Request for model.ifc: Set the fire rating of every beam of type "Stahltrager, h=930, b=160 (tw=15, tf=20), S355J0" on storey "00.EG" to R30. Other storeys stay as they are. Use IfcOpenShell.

First a look at what the model holds.

```python
import ifcopenshell
import ifcopenshell.util.element

model = ifcopenshell.open("model.ifc")
print(model.schema)
storey = next(s for s in model.by_type("IfcBuildingStorey") if s.Name == "00.EG")
beams = [e for e in ifcopenshell.util.element.get_decomposition(storey) if e.is_a("IfcBeam")]
seen = {}
for e in beams:
    element_type = ifcopenshell.util.element.get_type(e)
    key = (element_type.Name if element_type != e and element_type else None, ifcopenshell.util.element.get_pset(e, "Pset_BeamCommon", "FireRating"))
    seen[key] = seen.get(key, 0) + 1
for (name, value), count in sorted(seen.items(), key=str):
    print(count, "x", name, "|", value)
```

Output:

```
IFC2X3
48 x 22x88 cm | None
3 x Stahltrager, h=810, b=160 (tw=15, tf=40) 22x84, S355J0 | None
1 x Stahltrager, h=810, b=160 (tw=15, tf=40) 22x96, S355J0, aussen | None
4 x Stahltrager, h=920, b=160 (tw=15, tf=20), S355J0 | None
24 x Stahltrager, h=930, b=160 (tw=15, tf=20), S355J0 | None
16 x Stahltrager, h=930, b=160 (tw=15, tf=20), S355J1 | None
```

```python
import ifcopenshell
import ifcopenshell.api.pset
import ifcopenshell.util.element

model = ifcopenshell.open("model.ifc")

storey = next(s for s in model.by_type("IfcBuildingStorey") if s.Name == "00.EG")
beams = [e for e in ifcopenshell.util.element.get_decomposition(storey) if e.is_a("IfcBeam")]

count = 0
for e in beams:
    element_type = ifcopenshell.util.element.get_type(e)
    if element_type in (None, e) or element_type.Name != "Stahltrager, h=930, b=160 (tw=15, tf=20), S355J0":
        continue
    # add_pset returns the element's existing set when there is one.
    pset = ifcopenshell.api.pset.add_pset(model, product=e, name="Pset_BeamCommon")
    ifcopenshell.api.pset.edit_pset(model, pset=pset, properties={"FireRating": "R30"})
    count += 1

print(count, "beams updated")

model.write("model_edited.ifc")
```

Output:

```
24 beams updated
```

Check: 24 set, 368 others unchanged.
